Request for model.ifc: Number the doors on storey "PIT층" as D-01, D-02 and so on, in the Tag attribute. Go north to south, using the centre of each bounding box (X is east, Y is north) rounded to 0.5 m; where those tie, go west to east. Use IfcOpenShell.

First a look at what the model holds.

```python
import ifcopenshell
import ifcopenshell.util.element
import ifcopenshell.util.placement

model = ifcopenshell.open("model.ifc")
print(model.schema)
storey = next(s for s in model.by_type("IfcBuildingStorey") if s.Name == "PIT층")
doors = [e for e in ifcopenshell.util.element.get_decomposition(storey) if e.is_a("IfcDoor")]
for e in sorted(doors, key=lambda e: e.id()):
    origin = ifcopenshell.util.placement.get_local_placement(e.ObjectPlacement)[:3, 3]
    print(e.id(), e.Tag, e.Name, origin.round(2) + 0.0, sep=" | ")
```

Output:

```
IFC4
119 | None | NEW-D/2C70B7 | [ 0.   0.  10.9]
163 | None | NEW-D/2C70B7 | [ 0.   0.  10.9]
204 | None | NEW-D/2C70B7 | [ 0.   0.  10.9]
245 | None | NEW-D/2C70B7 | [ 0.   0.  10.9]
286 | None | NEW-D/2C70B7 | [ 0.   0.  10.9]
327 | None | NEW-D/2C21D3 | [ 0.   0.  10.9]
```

```python
import ifcopenshell
import ifcopenshell.geom
import ifcopenshell.util.element
import ifcopenshell.util.shape

model = ifcopenshell.open("model.ifc")
settings = ifcopenshell.geom.settings()
settings.set("use-world-coords", True)


def centre(element):
    shape = ifcopenshell.geom.create_shape(settings, element)
    return ifcopenshell.util.shape.get_bbox_centroid(shape.geometry)


storey = next(s for s in model.by_type("IfcBuildingStorey") if s.Name == "PIT층")
doors = [e for e in ifcopenshell.util.element.get_decomposition(storey) if e.is_a("IfcDoor")]

# Insertion points can sit at a corner or the storey origin, so sort by the geometry (in metres).
centres = {e: centre(e) for e in doors}
doors.sort(key=lambda e: (-round(centres[e][1] / 0.5), centres[e][0]))

for i, e in enumerate(doors, start=1):
    number = f"D-{i:02d}"
    e.Tag = number
    print(e.id(), number)

model.write("model-out.ifc")
```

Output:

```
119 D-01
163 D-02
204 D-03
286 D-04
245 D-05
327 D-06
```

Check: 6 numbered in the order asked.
